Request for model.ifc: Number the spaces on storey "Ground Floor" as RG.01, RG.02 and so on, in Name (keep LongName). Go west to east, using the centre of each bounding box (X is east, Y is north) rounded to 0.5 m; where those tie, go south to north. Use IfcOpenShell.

First a look at what the model holds.

```python
import ifcopenshell
import ifcopenshell.util.element
import ifcopenshell.util.placement

model = ifcopenshell.open("model.ifc")
print(model.schema)
storey = next(s for s in model.by_type("IfcBuildingStorey") if s.Name == "Ground Floor")
spaces = [e for e in ifcopenshell.util.element.get_decomposition(storey) if e.is_a("IfcSpace")]
for e in sorted(spaces, key=lambda e: e.id()):
    origin = ifcopenshell.util.placement.get_local_placement(e.ObjectPlacement)[:3, 3]
    print(e.id(), e.Name, e.LongName, origin.round(2) + 0.0, sep=" | ")
```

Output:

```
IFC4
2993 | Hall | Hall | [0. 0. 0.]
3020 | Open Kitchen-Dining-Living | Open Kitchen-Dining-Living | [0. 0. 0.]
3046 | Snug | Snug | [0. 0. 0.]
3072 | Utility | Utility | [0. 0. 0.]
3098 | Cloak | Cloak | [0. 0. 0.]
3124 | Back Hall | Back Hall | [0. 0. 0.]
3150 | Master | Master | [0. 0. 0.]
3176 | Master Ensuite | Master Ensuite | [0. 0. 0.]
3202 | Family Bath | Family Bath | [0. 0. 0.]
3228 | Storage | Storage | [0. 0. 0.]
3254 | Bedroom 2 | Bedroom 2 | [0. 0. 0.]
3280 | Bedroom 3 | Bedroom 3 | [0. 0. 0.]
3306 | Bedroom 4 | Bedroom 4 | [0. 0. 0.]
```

```python
import ifcopenshell
import ifcopenshell.geom
import ifcopenshell.util.element
import ifcopenshell.util.shape

model = ifcopenshell.open("model.ifc")
settings = ifcopenshell.geom.settings()
settings.set("use-world-coords", True)


def centre(element):
    shape = ifcopenshell.geom.create_shape(settings, element)
    return ifcopenshell.util.shape.get_bbox_centroid(shape.geometry)


storey = next(s for s in model.by_type("IfcBuildingStorey") if s.Name == "Ground Floor")
spaces = [e for e in ifcopenshell.util.element.get_decomposition(storey) if e.is_a("IfcSpace")]

# Insertion points can sit at a corner or the storey origin, so sort by the geometry (in metres).
centres = {e: centre(e) for e in spaces}
spaces.sort(key=lambda e: (round(centres[e][0] / 0.5), centres[e][1]))

for i, e in enumerate(spaces, start=1):
    number = f"RG.{i:02d}"
    e.Name = number
    print(e.id(), number)

model.write("model-out.ifc")
```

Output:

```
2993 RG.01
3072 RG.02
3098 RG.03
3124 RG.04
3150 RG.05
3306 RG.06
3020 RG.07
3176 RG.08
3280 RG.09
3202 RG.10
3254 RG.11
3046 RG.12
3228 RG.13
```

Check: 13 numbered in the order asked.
